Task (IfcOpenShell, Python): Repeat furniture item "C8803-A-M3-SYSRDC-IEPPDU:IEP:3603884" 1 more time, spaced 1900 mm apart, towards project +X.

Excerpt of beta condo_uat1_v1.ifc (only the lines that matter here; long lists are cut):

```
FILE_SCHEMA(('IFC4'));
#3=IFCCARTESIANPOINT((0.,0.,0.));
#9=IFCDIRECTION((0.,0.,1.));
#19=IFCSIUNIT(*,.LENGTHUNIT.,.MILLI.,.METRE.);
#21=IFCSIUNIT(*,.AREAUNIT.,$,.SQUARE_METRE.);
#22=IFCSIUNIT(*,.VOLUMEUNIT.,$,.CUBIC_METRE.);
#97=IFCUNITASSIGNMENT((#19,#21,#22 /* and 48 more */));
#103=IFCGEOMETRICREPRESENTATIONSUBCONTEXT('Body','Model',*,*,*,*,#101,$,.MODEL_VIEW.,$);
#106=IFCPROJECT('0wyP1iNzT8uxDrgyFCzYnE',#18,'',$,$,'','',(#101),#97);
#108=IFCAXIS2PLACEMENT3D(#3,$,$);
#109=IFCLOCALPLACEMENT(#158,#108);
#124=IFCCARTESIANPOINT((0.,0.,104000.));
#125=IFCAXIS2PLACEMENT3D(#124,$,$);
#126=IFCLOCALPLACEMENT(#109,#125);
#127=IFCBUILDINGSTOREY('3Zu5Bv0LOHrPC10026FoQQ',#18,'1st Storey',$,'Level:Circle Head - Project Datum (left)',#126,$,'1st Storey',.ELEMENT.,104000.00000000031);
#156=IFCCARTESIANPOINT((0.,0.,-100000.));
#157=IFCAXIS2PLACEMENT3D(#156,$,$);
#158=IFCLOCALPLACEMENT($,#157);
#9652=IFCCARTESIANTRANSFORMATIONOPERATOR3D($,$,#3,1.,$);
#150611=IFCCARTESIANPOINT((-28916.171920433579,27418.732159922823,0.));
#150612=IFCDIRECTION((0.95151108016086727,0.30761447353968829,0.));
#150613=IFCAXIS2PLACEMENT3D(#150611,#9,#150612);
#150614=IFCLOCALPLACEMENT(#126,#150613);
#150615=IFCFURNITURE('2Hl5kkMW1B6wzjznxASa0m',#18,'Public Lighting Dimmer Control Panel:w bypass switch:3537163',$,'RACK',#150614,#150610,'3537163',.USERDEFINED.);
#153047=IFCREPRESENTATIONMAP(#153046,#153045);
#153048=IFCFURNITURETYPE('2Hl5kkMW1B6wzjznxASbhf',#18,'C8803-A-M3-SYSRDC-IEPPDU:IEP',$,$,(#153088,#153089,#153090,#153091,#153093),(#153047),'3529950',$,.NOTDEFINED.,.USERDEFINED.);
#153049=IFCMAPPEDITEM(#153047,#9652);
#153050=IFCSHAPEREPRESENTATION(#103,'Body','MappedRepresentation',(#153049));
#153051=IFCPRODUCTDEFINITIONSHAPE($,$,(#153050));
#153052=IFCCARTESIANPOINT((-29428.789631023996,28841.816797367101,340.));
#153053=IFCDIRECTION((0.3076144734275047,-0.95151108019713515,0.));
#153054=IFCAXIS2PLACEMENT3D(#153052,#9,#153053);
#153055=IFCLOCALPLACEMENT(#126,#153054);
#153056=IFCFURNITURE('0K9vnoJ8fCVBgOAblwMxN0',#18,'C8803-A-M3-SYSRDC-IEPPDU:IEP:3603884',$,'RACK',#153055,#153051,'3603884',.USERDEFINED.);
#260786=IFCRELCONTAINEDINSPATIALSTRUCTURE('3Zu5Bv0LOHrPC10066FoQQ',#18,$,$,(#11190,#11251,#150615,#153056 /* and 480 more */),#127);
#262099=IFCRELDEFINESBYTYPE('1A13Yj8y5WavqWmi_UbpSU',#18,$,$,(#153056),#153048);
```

```python
import numpy as np
import ifcopenshell
import ifcopenshell.api.geometry
import ifcopenshell.api.root
import ifcopenshell.util.element
import ifcopenshell.util.placement

model = ifcopenshell.open("beta condo_uat1_v1.ifc")


def reuse_history(source, copy):
    """copy_class also copies each property set's owner history, people and application; keep the originals."""
    for rel in copy.IsDefinedBy:
        if rel.is_a("IfcRelDefinesByProperties") and (history := rel.RelatingPropertyDefinition.OwnerHistory):
            rel.RelatingPropertyDefinition.OwnerHistory = source.OwnerHistory
            ifcopenshell.util.element.remove_deep2(model, history)


source = model.by_guid("0K9vnoJ8fCVBgOAblwMxN0")
base = ifcopenshell.util.placement.get_local_placement(source.ObjectPlacement)
step = np.array([1.0, 0.0, 0.0]) * 1900.0

for i in range(1, 2):
    copy = ifcopenshell.api.root.copy_class(model, product=source)
    copy.Representation = ifcopenshell.util.element.copy_deep(
        model, source.Representation, exclude=["IfcGeometricRepresentationContext", "IfcRepresentationMap"]
    )
    copy.Name = "C8803-A-M3-SYSRDC-IEPPDU:IEP"
    copy.Tag = None
    reuse_history(source, copy)
    matrix = base.copy()
    matrix[:3, 3] += i * step
    print("added at", matrix[:3, 3].round(3) + 0.0)
    ifcopenshell.api.geometry.edit_object_placement(model, product=copy, matrix=matrix, is_si=False)

model.write("beta condo_uat1_v1_updated.ifc")
```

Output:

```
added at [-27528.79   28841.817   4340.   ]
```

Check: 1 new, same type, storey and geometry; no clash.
